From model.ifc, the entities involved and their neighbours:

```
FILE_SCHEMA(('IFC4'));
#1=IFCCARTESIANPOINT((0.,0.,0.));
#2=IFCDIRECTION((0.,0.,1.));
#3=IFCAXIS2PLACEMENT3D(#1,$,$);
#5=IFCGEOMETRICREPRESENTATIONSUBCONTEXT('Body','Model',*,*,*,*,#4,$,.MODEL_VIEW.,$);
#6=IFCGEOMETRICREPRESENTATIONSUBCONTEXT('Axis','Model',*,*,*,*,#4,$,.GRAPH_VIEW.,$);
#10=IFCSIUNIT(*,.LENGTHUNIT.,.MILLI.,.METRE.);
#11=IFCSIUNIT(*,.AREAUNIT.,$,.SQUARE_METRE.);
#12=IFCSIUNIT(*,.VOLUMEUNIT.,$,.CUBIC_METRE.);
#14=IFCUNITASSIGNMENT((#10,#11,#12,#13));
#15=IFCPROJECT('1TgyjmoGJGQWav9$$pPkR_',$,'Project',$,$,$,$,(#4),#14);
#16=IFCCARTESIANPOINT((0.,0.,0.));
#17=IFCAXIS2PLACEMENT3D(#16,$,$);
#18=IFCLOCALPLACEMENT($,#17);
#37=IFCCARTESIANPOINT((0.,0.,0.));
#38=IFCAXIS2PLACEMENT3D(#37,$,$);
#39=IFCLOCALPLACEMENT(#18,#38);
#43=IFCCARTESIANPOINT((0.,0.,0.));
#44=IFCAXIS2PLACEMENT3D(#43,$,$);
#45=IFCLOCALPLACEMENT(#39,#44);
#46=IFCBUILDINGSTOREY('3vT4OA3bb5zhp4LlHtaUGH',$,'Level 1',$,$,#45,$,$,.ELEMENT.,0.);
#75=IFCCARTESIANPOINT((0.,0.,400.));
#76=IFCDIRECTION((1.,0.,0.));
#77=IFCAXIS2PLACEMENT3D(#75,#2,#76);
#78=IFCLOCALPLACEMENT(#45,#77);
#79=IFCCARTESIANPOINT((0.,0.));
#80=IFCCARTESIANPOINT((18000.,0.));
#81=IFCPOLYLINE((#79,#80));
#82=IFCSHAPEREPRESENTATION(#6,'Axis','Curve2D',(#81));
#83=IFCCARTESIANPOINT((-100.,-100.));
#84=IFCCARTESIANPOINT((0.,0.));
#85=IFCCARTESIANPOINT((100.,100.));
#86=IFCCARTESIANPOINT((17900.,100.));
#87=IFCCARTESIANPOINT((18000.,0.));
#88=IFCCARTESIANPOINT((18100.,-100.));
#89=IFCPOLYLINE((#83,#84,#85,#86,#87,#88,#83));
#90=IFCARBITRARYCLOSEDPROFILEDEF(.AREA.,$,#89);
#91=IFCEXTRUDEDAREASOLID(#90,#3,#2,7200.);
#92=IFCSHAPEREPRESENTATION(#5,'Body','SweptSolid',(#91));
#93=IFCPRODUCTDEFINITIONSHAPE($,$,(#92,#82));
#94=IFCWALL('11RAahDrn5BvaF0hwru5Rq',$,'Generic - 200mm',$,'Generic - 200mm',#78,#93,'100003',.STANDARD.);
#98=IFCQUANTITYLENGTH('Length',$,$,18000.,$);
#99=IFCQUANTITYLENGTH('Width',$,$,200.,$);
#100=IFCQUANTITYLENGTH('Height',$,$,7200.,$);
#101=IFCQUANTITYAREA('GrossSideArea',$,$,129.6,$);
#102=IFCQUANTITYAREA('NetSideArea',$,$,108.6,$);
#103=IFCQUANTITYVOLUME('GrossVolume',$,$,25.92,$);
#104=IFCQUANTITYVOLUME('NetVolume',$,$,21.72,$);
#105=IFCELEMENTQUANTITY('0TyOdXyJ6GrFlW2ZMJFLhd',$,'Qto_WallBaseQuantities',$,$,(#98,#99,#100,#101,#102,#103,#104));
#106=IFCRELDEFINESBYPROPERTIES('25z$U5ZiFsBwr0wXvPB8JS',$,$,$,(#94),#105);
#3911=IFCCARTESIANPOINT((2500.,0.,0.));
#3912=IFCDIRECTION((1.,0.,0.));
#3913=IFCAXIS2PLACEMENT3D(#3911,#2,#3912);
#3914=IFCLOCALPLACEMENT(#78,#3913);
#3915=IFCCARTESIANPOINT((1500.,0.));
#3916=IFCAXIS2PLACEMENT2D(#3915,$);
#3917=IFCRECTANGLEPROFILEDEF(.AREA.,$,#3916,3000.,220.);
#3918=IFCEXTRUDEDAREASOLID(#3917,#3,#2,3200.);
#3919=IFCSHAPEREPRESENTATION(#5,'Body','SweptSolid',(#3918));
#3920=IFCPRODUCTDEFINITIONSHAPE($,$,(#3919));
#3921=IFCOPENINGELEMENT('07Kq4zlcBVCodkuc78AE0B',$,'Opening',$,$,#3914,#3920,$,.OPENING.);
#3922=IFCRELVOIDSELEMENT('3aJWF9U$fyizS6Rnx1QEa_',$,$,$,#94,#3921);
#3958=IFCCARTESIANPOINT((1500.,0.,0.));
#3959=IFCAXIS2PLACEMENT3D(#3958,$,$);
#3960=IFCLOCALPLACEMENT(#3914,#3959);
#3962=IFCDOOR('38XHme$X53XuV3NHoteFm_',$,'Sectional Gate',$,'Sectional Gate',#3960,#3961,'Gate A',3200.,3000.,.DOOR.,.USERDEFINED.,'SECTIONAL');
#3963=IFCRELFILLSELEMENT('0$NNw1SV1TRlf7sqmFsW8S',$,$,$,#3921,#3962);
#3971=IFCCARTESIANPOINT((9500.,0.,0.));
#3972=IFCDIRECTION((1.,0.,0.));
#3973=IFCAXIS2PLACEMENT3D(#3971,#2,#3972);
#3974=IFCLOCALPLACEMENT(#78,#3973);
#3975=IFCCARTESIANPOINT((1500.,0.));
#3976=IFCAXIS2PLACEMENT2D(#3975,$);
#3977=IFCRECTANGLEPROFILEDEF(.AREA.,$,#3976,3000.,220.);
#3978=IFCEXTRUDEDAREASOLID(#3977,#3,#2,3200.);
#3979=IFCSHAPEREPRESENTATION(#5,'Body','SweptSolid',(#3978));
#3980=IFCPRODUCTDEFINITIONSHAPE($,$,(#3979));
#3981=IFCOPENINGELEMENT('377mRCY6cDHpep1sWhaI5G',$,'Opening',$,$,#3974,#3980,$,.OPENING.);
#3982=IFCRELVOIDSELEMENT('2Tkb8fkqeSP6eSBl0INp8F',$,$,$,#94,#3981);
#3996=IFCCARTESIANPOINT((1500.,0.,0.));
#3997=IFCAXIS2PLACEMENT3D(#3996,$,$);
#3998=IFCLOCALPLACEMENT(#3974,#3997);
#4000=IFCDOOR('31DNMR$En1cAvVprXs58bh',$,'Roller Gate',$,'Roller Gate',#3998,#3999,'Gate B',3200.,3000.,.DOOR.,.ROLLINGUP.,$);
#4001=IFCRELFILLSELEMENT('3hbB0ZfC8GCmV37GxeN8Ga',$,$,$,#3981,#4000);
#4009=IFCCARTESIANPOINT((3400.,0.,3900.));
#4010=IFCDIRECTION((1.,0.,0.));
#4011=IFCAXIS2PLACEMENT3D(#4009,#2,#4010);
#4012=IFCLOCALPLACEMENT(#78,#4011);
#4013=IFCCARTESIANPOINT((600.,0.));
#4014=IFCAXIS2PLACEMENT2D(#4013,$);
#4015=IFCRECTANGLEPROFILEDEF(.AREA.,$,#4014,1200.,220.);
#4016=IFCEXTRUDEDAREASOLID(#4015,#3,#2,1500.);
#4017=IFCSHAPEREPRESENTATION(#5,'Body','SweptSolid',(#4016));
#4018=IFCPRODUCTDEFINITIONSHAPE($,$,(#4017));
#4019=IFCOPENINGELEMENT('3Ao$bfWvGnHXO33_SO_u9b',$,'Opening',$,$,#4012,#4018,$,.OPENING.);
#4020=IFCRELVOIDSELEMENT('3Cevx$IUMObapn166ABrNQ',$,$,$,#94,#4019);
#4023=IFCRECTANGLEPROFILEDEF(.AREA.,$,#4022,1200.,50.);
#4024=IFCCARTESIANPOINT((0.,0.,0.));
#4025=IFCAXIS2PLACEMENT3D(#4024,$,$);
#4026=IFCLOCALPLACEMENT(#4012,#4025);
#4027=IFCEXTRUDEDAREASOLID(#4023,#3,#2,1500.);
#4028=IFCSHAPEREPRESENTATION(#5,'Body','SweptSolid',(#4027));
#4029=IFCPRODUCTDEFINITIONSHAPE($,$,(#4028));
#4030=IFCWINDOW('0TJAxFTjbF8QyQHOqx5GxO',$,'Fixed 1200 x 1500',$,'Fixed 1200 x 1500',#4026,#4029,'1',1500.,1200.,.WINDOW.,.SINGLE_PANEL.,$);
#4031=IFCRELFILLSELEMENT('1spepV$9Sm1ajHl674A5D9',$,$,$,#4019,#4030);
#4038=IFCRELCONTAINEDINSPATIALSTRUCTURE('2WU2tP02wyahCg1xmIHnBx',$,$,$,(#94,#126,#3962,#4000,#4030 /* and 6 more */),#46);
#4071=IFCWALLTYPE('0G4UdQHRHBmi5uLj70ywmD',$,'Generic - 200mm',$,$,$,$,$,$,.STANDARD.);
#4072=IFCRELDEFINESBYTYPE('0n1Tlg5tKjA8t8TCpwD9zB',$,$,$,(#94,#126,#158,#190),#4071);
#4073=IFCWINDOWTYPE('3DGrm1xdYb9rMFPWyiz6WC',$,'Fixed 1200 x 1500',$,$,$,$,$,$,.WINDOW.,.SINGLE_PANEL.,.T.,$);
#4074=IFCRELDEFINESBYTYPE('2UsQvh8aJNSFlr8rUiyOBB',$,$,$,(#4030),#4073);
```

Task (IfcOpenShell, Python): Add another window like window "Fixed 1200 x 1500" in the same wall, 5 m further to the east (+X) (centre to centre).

```python
import ifcopenshell
import ifcopenshell.api.feature
import ifcopenshell.api.geometry
import ifcopenshell.api.pset
import ifcopenshell.api.root
import ifcopenshell.geom
import ifcopenshell.util.element
import ifcopenshell.util.placement
import ifcopenshell.util.shape
import ifcopenshell.util.unit

model = ifcopenshell.open("model.ifc")
unit_scale = ifcopenshell.util.unit.calculate_unit_scale(model)
area_scale = ifcopenshell.util.unit.calculate_unit_scale(model, "AREAUNIT")
volume_scale = ifcopenshell.util.unit.calculate_unit_scale(model, "VOLUMEUNIT")
settings = ifcopenshell.geom.settings()


def volume(element):
    """Net volume in cubic metres, openings subtracted."""
    shape = ifcopenshell.geom.create_shape(settings, element)
    return ifcopenshell.util.shape.get_volume(shape.geometry)


window = model.by_guid("0TJAxFTjbF8QyQHOqx5GxO")
opening = window.FillsVoids[0].RelatingOpeningElement
wall = opening.VoidsElements[0].RelatingBuildingElement
before = volume(wall)
shift = ifcopenshell.util.placement.get_local_placement(wall.ObjectPlacement)[:3, 0] * 5 / unit_scale

# copy_class copies the void relationship, type, container and properties, but no geometry.
new_opening = ifcopenshell.api.root.copy_class(model, product=opening)
new_opening.Representation = ifcopenshell.util.element.copy_deep(
    model, opening.Representation, exclude=["IfcGeometricRepresentationContext", "IfcRepresentationMap"]
)
new_window = ifcopenshell.api.root.copy_class(model, product=window)
new_window.Representation = ifcopenshell.util.element.copy_deep(
    model, window.Representation, exclude=["IfcGeometricRepresentationContext", "IfcRepresentationMap"]
)
new_window.Tag = None
ifcopenshell.api.feature.add_filling(model, opening=new_opening, element=new_window)

for old, new in ((opening, new_opening), (window, new_window)):
    matrix = ifcopenshell.util.placement.get_local_placement(old.ObjectPlacement)
    matrix[:3, 3] += shift
    ifcopenshell.api.geometry.edit_object_placement(model, product=new, matrix=matrix, is_si=False)

after = volume(wall)
thickness = 0.2  # wall thickness in metres

# Update the wall's stored quantities.
qto = model.by_id(ifcopenshell.util.element.get_pset(wall, "Qto_WallBaseQuantities", should_inherit=False)["id"])
ifcopenshell.api.pset.edit_qto(model, qto=qto, properties={
    "NetSideArea": after / thickness / area_scale,
    "NetVolume": after / volume_scale,
})

print(f"wall volume {before:.3f} -> {after:.3f} m3")

model.write("model_edited.ifc")
```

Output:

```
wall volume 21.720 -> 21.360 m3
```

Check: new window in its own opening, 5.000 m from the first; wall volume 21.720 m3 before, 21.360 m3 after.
